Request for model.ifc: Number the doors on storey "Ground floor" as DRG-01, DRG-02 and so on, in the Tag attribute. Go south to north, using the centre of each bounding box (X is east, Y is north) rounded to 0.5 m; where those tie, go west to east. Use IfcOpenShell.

First a look at what the model holds.

```python
import ifcopenshell
import ifcopenshell.util.element
import ifcopenshell.util.placement

model = ifcopenshell.open("model.ifc")
print(model.schema)
storey = next(s for s in model.by_type("IfcBuildingStorey") if s.Name == "Ground floor")
doors = [e for e in ifcopenshell.util.element.get_decomposition(storey) if e.is_a("IfcDoor")]
for e in sorted(doors, key=lambda e: e.id()):
    origin = ifcopenshell.util.placement.get_local_placement(e.ObjectPlacement)[:3, 3]
    print(e.id(), e.Tag, e.Name, origin.round(2) + 0.0, sep=" | ")
```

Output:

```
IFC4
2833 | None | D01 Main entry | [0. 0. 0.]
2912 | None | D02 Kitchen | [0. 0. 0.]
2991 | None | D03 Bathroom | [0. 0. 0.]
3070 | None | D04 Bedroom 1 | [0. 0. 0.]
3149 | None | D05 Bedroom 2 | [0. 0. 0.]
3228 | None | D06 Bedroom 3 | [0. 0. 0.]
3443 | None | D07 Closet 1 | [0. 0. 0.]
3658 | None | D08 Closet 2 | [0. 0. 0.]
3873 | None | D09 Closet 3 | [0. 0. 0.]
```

```python
import ifcopenshell
import ifcopenshell.geom
import ifcopenshell.util.element
import ifcopenshell.util.shape

model = ifcopenshell.open("model.ifc")
settings = ifcopenshell.geom.settings()
settings.set("use-world-coords", True)


def centre(element):
    shape = ifcopenshell.geom.create_shape(settings, element)
    return ifcopenshell.util.shape.get_bbox_centroid(shape.geometry)


storey = next(s for s in model.by_type("IfcBuildingStorey") if s.Name == "Ground floor")
doors = [e for e in ifcopenshell.util.element.get_decomposition(storey) if e.is_a("IfcDoor")]

# Insertion points can sit at a corner or the storey origin, so sort by the geometry (in metres).
centres = {e: centre(e) for e in doors}
doors.sort(key=lambda e: (round(centres[e][1] / 0.5), centres[e][0]))

for i, e in enumerate(doors, start=1):
    number = f"DRG-{i:02d}"
    e.Tag = number
    print(e.id(), number)

model.write("model_v2.ifc")
```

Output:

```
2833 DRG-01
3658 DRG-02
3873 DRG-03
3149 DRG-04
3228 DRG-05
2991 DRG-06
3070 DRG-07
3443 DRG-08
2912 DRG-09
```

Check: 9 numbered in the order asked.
